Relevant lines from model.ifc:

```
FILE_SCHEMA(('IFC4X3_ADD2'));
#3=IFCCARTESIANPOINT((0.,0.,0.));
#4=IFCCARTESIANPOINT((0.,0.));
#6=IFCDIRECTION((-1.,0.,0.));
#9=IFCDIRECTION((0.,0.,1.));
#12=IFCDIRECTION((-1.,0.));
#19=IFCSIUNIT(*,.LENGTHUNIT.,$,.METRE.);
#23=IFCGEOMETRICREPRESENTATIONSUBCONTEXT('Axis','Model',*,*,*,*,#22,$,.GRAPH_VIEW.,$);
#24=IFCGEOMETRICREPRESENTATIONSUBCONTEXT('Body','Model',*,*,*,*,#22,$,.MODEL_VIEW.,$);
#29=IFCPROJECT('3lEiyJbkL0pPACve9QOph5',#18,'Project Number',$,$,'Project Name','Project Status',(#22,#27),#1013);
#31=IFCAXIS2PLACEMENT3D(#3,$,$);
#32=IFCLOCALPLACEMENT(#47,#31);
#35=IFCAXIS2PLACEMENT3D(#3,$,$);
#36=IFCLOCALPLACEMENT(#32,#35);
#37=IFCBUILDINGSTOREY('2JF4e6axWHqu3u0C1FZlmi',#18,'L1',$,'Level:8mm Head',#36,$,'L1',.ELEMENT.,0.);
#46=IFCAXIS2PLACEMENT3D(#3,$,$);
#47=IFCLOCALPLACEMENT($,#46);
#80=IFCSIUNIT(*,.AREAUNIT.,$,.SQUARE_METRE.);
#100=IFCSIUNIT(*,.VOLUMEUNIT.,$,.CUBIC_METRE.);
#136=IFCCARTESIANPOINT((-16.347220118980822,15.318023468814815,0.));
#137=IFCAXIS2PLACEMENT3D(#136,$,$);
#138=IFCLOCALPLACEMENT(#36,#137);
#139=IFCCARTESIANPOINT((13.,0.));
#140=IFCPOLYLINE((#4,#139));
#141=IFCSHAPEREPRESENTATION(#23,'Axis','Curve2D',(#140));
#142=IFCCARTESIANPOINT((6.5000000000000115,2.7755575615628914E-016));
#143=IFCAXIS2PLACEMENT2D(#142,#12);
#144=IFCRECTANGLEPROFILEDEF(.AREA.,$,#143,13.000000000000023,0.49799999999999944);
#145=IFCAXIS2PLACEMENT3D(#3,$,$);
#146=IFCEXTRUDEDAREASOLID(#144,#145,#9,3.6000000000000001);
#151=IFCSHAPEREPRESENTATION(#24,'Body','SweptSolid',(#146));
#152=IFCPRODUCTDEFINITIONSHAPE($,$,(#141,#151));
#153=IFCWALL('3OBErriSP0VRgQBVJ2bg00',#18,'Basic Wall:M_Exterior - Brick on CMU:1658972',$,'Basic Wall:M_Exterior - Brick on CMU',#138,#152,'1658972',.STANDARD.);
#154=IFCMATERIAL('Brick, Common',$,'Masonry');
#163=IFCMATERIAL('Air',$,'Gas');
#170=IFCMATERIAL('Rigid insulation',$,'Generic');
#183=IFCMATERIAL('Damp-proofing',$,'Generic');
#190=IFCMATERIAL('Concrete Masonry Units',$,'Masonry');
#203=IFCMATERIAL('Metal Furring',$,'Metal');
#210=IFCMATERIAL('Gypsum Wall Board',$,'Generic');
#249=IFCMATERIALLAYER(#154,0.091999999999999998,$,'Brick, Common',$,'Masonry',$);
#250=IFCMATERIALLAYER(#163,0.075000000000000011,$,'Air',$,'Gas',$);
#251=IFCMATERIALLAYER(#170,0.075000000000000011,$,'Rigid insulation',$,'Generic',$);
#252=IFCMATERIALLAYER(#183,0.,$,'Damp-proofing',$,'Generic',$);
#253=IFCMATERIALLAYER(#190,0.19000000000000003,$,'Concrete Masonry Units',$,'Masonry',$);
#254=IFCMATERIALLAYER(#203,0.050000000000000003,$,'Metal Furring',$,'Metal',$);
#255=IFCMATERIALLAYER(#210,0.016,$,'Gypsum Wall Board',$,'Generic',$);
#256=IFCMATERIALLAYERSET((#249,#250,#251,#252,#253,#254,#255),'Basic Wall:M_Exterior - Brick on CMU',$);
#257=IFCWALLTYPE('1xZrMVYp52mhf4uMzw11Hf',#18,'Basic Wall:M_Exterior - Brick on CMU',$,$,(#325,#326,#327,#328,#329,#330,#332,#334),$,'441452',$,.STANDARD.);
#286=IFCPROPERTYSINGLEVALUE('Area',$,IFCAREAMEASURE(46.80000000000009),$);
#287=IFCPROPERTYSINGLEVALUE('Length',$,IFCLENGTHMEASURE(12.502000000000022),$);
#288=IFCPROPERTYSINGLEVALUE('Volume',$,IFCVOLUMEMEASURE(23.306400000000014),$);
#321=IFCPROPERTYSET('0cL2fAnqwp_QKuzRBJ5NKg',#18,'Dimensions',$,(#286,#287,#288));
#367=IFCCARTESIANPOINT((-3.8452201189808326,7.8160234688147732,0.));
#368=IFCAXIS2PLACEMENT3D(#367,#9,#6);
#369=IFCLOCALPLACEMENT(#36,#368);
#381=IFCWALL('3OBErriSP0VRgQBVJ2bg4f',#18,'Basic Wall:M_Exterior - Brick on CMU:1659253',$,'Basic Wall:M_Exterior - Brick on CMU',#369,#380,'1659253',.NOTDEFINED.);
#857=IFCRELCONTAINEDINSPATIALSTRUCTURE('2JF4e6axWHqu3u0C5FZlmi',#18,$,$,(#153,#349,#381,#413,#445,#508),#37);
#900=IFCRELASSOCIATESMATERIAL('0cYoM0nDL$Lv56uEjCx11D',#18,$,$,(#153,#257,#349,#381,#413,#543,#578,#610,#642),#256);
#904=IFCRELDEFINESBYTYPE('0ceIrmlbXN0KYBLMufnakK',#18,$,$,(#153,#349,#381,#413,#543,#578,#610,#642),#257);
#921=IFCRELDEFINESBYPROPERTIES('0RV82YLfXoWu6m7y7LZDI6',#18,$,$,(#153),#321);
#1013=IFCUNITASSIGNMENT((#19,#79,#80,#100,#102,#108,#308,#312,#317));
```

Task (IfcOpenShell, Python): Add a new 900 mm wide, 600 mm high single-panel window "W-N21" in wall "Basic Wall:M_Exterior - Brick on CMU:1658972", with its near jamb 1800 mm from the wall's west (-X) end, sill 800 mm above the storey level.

```python
import numpy as np
import ifcopenshell
import ifcopenshell.api.feature
import ifcopenshell.api.geometry
import ifcopenshell.api.pset
import ifcopenshell.api.root
import ifcopenshell.api.spatial
import ifcopenshell.geom
import ifcopenshell.util.element
import ifcopenshell.util.placement
import ifcopenshell.util.representation
import ifcopenshell.util.shape
import ifcopenshell.util.unit

model = ifcopenshell.open("model.ifc")
unit_scale = ifcopenshell.util.unit.calculate_unit_scale(model)
area_scale = ifcopenshell.util.unit.calculate_unit_scale(model, "AREAUNIT")
volume_scale = ifcopenshell.util.unit.calculate_unit_scale(model, "VOLUMEUNIT")
settings = ifcopenshell.geom.settings()


def volume(element):
    """Net volume in cubic metres, openings subtracted."""
    shape = ifcopenshell.geom.create_shape(settings, element)
    return ifcopenshell.util.shape.get_volume(shape.geometry)


wall = model.by_guid("3OBErriSP0VRgQBVJ2bg00")
storey = ifcopenshell.util.element.get_container(wall, ifc_class="IfcBuildingStorey")
context = ifcopenshell.util.representation.get_context(model, "Model", "Body", "MODEL_VIEW")
before = volume(wall)

width, height, from_end, sill = 0.9, 0.6, 1.8, 0.8  # metres

# The wall runs along its own X axis, and the end named is its -X end.
wall_shape = ifcopenshell.geom.create_shape(settings, wall)
x, y, z = ifcopenshell.util.shape.get_vertices(wall_shape.geometry).T
start = x.min() + from_end
face, thickness = float(y.min()), float(y.max() - y.min())
wall_matrix = ifcopenshell.util.placement.get_local_placement(wall.ObjectPlacement)
level = ifcopenshell.util.placement.get_local_placement(storey.ObjectPlacement)[2, 3]


def in_wall(x, y):
    """Placement at x, y metres in the wall's axes, at sill height."""
    matrix = wall_matrix.copy()
    matrix[:, 3] = wall_matrix @ np.array([x / unit_scale, y / unit_scale, 0.0, 1.0])
    matrix[2, 3] = level + sill / unit_scale
    return matrix


# Opening: a box that overshoots both wall faces by 50 mm.
opening = ifcopenshell.api.root.create_entity(model, ifc_class="IfcOpeningElement", predefined_type="OPENING")
box = ifcopenshell.api.geometry.add_wall_representation(
    model, context=context, length=width, height=height, thickness=thickness + 0.1
)
ifcopenshell.api.geometry.assign_representation(model, product=opening, representation=box)
ifcopenshell.api.geometry.edit_object_placement(model, product=opening, matrix=in_wall(start, face - 0.05), is_si=False)
ifcopenshell.api.feature.add_feature(model, feature=opening, element=wall)

window = ifcopenshell.api.root.create_entity(model, ifc_class="IfcWindow", name="W-N21", predefined_type="WINDOW")
window.OverallWidth, window.OverallHeight = width / unit_scale, height / unit_scale
window.PartitioningType = "SINGLE_PANEL"
body = ifcopenshell.api.geometry.add_window_representation(
    model,
    context=context,
    overall_width=window.OverallWidth,
    overall_height=window.OverallHeight,
    partition_type="SINGLE_PANEL",
)
ifcopenshell.api.geometry.assign_representation(model, product=window, representation=body)
ifcopenshell.api.spatial.assign_container(model, products=[window], relating_structure=storey)
ifcopenshell.api.feature.add_filling(model, opening=opening, element=window)

# Centre the window in the wall's thickness.
ifcopenshell.api.geometry.edit_object_placement(model, product=window, matrix=in_wall(start, face), is_si=False)
window_shape = ifcopenshell.geom.create_shape(settings, window)
depth = ifcopenshell.util.shape.get_vertices(window_shape.geometry)[:, 1]
offset = face + thickness / 2 - (depth.min() + depth.max()) / 2
ifcopenshell.api.geometry.edit_object_placement(model, product=window, matrix=in_wall(start, offset), is_si=False)

after = volume(wall)

# Update the wall's stored quantities.
pset = model.by_id(ifcopenshell.util.element.get_pset(wall, "Dimensions", should_inherit=False)["id"])
ifcopenshell.api.pset.edit_pset(model, pset=pset, properties={
    "Area": model.create_entity("IfcAreaMeasure", after / thickness / area_scale),
    "Volume": model.create_entity("IfcVolumeMeasure", after / volume_scale),
})

print(f"wall volume {before:.3f} -> {after:.3f} m3")

model.write("model-out.ifc")
```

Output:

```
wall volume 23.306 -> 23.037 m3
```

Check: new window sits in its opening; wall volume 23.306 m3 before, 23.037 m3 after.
